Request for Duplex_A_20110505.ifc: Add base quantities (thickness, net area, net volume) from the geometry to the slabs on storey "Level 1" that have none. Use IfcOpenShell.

First a look at what the model holds.

```python
import ifcopenshell
import ifcopenshell.util.element
import ifcopenshell.util.unit

model = ifcopenshell.open("Duplex_A_20110505.ifc")
print(model.schema)
for unit_type in ("LENGTHUNIT", "AREAUNIT", "VOLUMEUNIT"):
    print(unit_type, ifcopenshell.util.unit.calculate_unit_scale(model, unit_type))
storey = next(s for s in model.by_type("IfcBuildingStorey") if s.Name == "Level 1")
slabs = [e for e in ifcopenshell.util.element.get_decomposition(storey) if e.is_a("IfcSlab")]
for e in sorted(slabs, key=lambda e: e.id()):
    print(e.id(), e.is_a(), e.Name, list(ifcopenshell.util.element.get_psets(e, qtos_only=True)), sep=" | ")
```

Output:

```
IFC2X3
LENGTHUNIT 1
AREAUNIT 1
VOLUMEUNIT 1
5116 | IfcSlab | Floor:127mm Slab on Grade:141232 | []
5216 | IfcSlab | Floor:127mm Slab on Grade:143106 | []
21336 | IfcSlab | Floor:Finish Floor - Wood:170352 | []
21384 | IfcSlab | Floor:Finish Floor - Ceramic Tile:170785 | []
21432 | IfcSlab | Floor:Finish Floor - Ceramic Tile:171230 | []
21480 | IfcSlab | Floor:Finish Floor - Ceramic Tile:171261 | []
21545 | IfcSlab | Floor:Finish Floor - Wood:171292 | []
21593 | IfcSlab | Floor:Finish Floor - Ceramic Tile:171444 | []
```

```python
import ifcopenshell
import ifcopenshell.api.pset
import ifcopenshell.geom
import ifcopenshell.util.element
import ifcopenshell.util.shape
import ifcopenshell.util.unit

model = ifcopenshell.open("Duplex_A_20110505.ifc")
unit_scale = ifcopenshell.util.unit.calculate_unit_scale(model)
area_scale = ifcopenshell.util.unit.calculate_unit_scale(model, "AREAUNIT")
volume_scale = ifcopenshell.util.unit.calculate_unit_scale(model, "VOLUMEUNIT")
settings = ifcopenshell.geom.settings()

storey = next(s for s in model.by_type("IfcBuildingStorey") if s.Name == "Level 1")
slabs = [e for e in ifcopenshell.util.element.get_decomposition(storey) if e.is_a("IfcSlab")]

for e in sorted(slabs, key=lambda e: e.id()):
    if ifcopenshell.util.element.get_psets(e, qtos_only=True, should_inherit=False):
        continue
    # Geometry comes back in metres, in the element's own axes.
    shape = ifcopenshell.geom.create_shape(settings, e)
    values = {
        "Width": ifcopenshell.util.shape.get_z(shape.geometry) / unit_scale,
        "NetArea": ifcopenshell.util.shape.get_footprint_area(shape.geometry) / area_scale,
        "NetVolume": ifcopenshell.util.shape.get_volume(shape.geometry) / volume_scale,
    }
    qto = ifcopenshell.api.pset.add_qto(model, product=e, name="BaseQuantities")
    ifcopenshell.api.pset.edit_qto(model, qto=qto, properties=values)
    print(e.id(), {k: round(v, 3) for k, v in values.items()})

model.write("Duplex_A_20110505_v2.ifc")
```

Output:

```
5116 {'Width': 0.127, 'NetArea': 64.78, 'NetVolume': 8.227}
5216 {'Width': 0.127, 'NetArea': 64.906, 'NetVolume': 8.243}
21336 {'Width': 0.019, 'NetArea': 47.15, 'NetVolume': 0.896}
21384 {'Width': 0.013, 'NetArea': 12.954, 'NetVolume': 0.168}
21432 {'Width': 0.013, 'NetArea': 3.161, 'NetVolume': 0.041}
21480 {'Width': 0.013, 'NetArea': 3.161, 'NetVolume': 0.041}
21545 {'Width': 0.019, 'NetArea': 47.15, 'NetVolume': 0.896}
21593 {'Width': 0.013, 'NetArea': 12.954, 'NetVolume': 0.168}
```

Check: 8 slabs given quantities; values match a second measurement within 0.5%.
